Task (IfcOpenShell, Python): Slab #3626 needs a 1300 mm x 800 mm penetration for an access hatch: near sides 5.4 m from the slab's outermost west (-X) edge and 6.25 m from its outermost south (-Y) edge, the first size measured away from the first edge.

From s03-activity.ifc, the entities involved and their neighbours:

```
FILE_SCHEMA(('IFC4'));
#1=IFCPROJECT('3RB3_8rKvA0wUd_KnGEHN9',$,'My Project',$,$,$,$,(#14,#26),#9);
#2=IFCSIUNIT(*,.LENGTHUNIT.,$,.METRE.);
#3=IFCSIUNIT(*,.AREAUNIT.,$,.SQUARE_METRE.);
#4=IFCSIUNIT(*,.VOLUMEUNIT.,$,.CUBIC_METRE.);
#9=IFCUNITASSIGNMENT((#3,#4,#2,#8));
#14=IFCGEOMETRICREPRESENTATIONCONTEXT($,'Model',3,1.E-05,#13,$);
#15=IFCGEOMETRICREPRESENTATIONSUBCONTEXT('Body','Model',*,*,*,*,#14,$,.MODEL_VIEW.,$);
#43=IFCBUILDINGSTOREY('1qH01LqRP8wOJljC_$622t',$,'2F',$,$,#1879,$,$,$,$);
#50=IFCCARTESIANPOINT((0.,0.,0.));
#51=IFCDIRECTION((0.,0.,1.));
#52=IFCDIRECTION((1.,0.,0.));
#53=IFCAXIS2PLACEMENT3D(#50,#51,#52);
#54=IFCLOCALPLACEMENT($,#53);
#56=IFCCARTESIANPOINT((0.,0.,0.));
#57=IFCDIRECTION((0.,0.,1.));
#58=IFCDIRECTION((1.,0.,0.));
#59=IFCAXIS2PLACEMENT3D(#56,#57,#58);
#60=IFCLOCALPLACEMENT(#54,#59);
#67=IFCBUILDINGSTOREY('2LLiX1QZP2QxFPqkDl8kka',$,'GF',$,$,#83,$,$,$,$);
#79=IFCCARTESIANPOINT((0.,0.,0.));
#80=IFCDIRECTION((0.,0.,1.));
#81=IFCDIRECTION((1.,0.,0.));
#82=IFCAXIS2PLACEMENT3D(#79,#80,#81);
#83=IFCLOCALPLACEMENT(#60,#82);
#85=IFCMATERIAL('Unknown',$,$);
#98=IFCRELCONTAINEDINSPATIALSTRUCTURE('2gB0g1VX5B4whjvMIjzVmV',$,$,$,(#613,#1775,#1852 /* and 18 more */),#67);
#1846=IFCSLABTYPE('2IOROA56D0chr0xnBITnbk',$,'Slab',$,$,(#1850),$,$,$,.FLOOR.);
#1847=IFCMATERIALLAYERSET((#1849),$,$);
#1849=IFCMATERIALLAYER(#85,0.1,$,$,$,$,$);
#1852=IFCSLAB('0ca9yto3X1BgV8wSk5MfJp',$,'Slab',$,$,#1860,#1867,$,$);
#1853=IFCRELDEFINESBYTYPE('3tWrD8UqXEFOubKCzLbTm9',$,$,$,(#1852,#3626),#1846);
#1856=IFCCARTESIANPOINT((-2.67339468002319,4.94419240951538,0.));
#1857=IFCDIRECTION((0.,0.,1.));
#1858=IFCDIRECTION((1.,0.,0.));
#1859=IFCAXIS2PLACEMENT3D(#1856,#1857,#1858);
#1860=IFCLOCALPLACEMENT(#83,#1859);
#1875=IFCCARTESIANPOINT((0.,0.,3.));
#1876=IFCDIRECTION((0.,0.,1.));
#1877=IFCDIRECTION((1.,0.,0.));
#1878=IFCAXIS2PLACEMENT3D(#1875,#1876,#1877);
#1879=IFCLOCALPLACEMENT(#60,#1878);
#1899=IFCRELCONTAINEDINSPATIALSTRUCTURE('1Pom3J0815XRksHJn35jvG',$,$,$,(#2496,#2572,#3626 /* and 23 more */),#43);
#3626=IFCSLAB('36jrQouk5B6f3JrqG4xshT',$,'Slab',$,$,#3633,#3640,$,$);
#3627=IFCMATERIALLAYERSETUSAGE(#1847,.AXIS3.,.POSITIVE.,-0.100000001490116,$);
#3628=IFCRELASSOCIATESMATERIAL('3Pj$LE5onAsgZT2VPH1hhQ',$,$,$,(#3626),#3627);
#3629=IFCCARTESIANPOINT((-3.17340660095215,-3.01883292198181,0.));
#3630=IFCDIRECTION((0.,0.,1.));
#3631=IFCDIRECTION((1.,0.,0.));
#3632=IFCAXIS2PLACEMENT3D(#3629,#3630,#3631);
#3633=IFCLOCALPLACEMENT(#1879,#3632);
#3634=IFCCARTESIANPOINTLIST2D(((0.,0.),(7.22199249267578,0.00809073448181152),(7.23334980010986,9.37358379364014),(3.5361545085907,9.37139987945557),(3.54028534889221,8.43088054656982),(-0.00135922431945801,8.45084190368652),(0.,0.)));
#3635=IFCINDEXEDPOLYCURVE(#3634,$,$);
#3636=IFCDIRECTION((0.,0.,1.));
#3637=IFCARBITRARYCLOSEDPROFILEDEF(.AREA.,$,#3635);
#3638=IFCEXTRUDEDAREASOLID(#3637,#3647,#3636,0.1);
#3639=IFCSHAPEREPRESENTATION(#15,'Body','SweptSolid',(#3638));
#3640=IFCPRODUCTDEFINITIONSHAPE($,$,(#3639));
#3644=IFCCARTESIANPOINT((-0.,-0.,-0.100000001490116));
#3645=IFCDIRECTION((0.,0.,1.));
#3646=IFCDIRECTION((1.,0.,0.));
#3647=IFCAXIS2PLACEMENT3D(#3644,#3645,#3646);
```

```python
import numpy as np
import ifcopenshell
import ifcopenshell.api.feature
import ifcopenshell.api.geometry
import ifcopenshell.api.root
import ifcopenshell.geom
import ifcopenshell.util.placement
import ifcopenshell.util.representation
import ifcopenshell.util.shape
import ifcopenshell.util.unit

model = ifcopenshell.open("s03-activity.ifc")
unit_scale = ifcopenshell.util.unit.calculate_unit_scale(model)
settings = ifcopenshell.geom.settings()


def volume(element):
    """Net volume in cubic metres, openings subtracted."""
    shape = ifcopenshell.geom.create_shape(settings, element)
    return ifcopenshell.util.shape.get_volume(shape.geometry)


slab = model.by_id(3626)
before = volume(slab)

# Extent in the slab's own axes, in metres. The edges named are its -X and -Y sides.
slab_shape = ifcopenshell.geom.create_shape(settings, slab)
vertices = ifcopenshell.util.shape.get_vertices(slab_shape.geometry)
x_min, y_min, bottom = vertices.min(axis=0)
top = vertices[:, 2].max()

opening = ifcopenshell.api.root.create_entity(model, ifc_class="IfcOpeningElement", name="Access hatch opening", predefined_type="OPENING")
context = ifcopenshell.util.representation.get_context(model, "Model", "Body", "MODEL_VIEW")
width, depth = 1.3, 0.8
outline = [(0.0, 0.0), (width, 0.0), (width, depth), (0.0, depth), (0.0, 0.0)]
# Overshoot both faces by 50 mm so the cut is clean.
shape = ifcopenshell.api.geometry.add_slab_representation(
    model, context=context, depth=top - bottom + 0.1, polyline=outline
)
ifcopenshell.api.geometry.assign_representation(model, product=opening, representation=shape)

matrix = ifcopenshell.util.placement.get_local_placement(slab.ObjectPlacement)
matrix[:, 3] = matrix @ np.append(np.array([x_min + 5.4, y_min + 6.25, bottom - 0.05]) / unit_scale, 1.0)
ifcopenshell.api.geometry.edit_object_placement(model, product=opening, matrix=matrix, is_si=False)
ifcopenshell.api.feature.add_feature(model, feature=opening, element=slab)

after = volume(slab)

print(f"slab volume {before:.3f} -> {after:.3f} m3")

model.write("s03-activity_rev.ifc")
```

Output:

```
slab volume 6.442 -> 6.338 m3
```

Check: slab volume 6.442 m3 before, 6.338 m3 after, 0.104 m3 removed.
